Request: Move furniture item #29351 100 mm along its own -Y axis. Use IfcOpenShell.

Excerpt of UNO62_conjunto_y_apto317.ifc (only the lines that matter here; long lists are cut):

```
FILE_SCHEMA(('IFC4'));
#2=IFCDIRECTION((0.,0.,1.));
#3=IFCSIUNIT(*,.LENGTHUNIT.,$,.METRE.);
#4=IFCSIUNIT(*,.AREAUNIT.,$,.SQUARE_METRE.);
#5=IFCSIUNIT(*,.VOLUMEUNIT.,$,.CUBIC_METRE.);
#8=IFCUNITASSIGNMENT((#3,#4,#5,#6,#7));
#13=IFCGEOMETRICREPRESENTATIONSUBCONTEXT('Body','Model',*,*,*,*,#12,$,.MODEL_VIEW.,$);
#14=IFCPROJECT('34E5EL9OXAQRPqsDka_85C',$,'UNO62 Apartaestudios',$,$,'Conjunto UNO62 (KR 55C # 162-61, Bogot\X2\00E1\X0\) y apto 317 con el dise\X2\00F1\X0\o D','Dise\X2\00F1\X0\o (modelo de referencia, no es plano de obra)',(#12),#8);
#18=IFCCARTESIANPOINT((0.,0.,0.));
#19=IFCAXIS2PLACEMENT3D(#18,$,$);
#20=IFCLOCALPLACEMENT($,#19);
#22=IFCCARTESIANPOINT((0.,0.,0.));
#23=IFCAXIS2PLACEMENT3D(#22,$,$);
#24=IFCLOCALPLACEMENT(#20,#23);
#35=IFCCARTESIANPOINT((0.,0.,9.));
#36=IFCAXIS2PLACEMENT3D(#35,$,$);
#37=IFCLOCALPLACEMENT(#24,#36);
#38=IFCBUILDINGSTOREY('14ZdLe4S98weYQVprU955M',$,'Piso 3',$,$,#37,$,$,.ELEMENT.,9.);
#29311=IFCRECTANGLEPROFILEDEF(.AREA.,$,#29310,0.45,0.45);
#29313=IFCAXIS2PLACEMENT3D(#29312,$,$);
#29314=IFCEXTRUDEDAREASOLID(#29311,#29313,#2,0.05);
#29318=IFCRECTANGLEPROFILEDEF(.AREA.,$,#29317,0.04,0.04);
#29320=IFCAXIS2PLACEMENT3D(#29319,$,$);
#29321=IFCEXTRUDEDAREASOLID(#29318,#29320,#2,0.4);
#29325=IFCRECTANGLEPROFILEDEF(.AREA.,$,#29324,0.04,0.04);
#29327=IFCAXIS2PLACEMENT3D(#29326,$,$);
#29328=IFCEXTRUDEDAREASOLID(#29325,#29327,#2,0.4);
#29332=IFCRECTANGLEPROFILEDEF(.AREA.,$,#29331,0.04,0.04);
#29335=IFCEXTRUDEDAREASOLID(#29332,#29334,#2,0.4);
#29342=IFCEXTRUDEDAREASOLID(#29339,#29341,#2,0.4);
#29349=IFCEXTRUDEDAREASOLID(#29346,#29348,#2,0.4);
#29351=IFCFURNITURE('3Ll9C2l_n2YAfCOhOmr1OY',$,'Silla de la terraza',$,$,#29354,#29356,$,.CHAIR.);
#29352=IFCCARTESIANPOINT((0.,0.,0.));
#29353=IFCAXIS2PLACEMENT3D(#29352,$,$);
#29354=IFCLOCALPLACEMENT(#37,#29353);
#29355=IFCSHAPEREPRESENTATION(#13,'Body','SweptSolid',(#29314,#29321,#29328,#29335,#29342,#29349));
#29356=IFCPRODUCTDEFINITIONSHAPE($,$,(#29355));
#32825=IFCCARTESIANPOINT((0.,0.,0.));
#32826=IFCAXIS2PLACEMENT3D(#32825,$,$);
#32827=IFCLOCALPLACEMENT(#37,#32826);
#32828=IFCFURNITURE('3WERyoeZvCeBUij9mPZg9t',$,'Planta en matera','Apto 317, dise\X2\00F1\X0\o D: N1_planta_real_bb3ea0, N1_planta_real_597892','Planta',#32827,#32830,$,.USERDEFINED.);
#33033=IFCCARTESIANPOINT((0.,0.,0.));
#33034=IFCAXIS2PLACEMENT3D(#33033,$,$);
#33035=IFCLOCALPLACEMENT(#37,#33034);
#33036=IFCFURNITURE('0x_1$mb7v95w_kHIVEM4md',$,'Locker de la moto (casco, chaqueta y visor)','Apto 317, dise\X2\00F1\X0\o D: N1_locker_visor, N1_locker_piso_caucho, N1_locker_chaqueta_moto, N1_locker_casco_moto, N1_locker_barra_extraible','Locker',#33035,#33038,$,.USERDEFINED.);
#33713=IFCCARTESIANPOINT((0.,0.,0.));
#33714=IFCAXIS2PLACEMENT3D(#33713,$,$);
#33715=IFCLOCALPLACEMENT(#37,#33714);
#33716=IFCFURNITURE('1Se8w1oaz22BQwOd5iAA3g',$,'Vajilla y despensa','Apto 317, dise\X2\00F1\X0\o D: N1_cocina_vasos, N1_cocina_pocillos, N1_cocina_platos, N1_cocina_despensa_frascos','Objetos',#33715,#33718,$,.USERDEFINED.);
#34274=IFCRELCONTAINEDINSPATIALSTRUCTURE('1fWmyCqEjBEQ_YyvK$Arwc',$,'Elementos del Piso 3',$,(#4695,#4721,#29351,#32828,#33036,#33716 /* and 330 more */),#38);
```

```python
import ifcopenshell
import ifcopenshell.api.geometry
import ifcopenshell.util.placement
import ifcopenshell.util.unit

model = ifcopenshell.open("UNO62_conjunto_y_apto317.ifc")
unit_scale = ifcopenshell.util.unit.calculate_unit_scale(model)

item = model.by_guid("3Ll9C2l_n2YAfCOhOmr1OY")
matrix = ifcopenshell.util.placement.get_local_placement(item.ObjectPlacement)
matrix[:3, 3] -= matrix[:3, 1] * 0.1 / unit_scale
ifcopenshell.api.geometry.edit_object_placement(model, product=item, matrix=matrix, is_si=False)

print(ifcopenshell.util.placement.get_local_placement(item.ObjectPlacement).round(3) + 0.0)

model.write("UNO62_conjunto_y_apto317_rev.ifc")
```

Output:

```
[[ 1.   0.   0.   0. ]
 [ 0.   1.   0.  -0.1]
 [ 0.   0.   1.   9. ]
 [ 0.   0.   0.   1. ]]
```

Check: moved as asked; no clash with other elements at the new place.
